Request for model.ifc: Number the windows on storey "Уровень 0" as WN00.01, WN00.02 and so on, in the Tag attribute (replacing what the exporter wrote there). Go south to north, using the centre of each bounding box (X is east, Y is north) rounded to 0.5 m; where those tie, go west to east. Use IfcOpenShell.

First a look at what the model holds.

```python
import ifcopenshell
import ifcopenshell.util.element
import ifcopenshell.util.placement

model = ifcopenshell.open("model.ifc")
print(model.schema)
storey = next(s for s in model.by_type("IfcBuildingStorey") if s.Name == "Уровень 0")
windows = [e for e in ifcopenshell.util.element.get_decomposition(storey) if e.is_a("IfcWindow")]
for e in sorted(windows, key=lambda e: e.id()):
    origin = ifcopenshell.util.placement.get_local_placement(e.ObjectPlacement)[:3, 3]
    print(e.id(), e.Tag, e.Name, origin.round(2) + 0.0, sep=" | ")
```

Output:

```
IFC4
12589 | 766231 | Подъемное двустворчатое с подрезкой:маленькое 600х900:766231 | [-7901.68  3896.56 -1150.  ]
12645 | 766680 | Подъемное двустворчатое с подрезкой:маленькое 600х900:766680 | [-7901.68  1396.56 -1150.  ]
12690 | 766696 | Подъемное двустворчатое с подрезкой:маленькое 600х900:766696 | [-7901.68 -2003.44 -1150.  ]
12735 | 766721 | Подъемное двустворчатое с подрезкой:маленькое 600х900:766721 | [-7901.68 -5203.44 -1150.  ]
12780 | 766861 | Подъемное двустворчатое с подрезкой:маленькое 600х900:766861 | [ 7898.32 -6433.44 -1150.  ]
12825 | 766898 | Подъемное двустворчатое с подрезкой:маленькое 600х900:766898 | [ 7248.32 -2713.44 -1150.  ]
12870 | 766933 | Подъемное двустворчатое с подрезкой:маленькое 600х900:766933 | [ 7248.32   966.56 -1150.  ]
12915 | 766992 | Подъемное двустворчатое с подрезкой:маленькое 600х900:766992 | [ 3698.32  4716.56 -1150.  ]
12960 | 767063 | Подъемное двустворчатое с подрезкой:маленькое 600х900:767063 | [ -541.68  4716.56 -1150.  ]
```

```python
import ifcopenshell
import ifcopenshell.geom
import ifcopenshell.util.element
import ifcopenshell.util.shape

model = ifcopenshell.open("model.ifc")
settings = ifcopenshell.geom.settings()
settings.set("use-world-coords", True)


def centre(element):
    shape = ifcopenshell.geom.create_shape(settings, element)
    return ifcopenshell.util.shape.get_bbox_centroid(shape.geometry)


storey = next(s for s in model.by_type("IfcBuildingStorey") if s.Name == "Уровень 0")
windows = [e for e in ifcopenshell.util.element.get_decomposition(storey) if e.is_a("IfcWindow")]

# Insertion points can sit at a corner or the storey origin, so sort by the geometry (in metres).
centres = {e: centre(e) for e in windows}
windows.sort(key=lambda e: (round(centres[e][1] / 0.5), centres[e][0]))

for i, e in enumerate(windows, start=1):
    number = f"WN00.{i:02d}"
    e.Tag = number
    print(e.id(), number)

model.write("model_updated.ifc")
```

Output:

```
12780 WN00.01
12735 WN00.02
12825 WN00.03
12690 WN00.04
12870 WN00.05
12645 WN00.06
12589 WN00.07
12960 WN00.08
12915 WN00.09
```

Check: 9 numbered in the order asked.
